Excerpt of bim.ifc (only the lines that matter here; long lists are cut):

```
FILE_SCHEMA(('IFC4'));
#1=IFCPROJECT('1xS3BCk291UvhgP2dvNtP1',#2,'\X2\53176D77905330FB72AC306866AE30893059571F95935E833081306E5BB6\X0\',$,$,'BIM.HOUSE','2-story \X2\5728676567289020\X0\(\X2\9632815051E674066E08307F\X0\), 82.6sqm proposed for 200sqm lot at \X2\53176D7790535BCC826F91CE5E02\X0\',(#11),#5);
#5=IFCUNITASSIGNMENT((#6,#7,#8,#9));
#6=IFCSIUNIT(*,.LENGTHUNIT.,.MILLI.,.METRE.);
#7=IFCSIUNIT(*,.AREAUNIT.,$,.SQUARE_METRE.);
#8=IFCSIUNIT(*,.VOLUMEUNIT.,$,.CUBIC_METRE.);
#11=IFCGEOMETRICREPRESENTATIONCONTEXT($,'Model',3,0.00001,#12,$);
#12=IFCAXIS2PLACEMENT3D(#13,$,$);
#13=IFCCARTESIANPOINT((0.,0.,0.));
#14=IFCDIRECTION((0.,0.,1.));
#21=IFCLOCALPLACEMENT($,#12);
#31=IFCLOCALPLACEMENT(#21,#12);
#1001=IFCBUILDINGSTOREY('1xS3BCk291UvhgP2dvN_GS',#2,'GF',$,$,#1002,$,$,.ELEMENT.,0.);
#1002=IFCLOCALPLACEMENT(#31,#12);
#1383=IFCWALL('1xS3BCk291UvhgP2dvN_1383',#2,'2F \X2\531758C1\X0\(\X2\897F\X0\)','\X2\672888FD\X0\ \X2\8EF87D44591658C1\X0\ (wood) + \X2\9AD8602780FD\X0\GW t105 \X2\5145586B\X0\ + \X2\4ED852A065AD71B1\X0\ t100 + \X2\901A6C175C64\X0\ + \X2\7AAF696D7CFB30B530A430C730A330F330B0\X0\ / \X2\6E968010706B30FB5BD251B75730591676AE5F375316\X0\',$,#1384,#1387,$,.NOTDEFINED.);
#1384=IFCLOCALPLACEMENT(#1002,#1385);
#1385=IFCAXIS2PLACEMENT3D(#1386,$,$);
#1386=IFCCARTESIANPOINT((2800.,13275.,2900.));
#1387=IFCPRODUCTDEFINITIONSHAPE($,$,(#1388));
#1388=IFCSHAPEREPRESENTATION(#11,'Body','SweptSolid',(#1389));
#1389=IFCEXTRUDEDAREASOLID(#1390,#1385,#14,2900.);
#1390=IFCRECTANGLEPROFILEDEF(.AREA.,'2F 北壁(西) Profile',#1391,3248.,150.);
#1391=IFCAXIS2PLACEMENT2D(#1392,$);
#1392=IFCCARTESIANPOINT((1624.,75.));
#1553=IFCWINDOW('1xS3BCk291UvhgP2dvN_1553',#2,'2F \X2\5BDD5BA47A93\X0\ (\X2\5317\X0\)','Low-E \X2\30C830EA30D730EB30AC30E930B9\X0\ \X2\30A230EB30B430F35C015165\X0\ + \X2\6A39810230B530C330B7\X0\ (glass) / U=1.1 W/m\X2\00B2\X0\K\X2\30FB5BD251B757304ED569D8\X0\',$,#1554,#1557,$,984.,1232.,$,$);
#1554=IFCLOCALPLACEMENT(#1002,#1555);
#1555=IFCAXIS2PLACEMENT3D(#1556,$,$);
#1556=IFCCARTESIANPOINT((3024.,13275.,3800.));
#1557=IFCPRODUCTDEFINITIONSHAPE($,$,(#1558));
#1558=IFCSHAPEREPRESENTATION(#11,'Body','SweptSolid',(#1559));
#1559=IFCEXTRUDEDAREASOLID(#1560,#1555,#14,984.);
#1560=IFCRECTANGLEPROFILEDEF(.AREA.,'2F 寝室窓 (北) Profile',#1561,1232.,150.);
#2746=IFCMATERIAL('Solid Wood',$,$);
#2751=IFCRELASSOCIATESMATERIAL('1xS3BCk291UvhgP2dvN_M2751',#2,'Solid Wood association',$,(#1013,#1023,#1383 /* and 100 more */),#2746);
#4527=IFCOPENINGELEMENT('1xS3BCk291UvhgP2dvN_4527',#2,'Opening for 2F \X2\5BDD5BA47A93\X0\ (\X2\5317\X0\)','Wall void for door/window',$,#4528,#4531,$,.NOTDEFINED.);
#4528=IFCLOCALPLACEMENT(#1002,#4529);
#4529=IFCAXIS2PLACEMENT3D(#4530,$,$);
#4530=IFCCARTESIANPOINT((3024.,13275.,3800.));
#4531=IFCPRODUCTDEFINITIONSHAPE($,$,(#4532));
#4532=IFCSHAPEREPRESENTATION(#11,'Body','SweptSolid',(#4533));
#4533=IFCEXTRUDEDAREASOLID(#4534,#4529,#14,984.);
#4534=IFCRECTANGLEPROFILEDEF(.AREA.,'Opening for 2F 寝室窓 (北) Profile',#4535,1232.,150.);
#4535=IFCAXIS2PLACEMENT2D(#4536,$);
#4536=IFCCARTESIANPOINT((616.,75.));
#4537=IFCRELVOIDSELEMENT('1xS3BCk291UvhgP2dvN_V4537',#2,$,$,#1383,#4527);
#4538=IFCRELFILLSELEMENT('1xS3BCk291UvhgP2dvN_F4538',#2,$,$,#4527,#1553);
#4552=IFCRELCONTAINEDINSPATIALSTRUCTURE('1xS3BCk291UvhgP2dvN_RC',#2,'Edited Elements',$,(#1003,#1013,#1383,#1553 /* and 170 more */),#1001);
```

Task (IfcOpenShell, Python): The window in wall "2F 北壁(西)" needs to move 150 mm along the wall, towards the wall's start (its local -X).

```python
import ifcopenshell
import ifcopenshell.api.geometry
import ifcopenshell.util.placement
import ifcopenshell.util.unit

model = ifcopenshell.open("bim.ifc")
unit_scale = ifcopenshell.util.unit.calculate_unit_scale(model)

window = model.by_id(1553)
opening = window.FillsVoids[0].RelatingOpeningElement
wall = opening.VoidsElements[0].RelatingBuildingElement

wall_matrix = ifcopenshell.util.placement.get_local_placement(wall.ObjectPlacement)
shift = wall_matrix[:3, 0] * -0.15 / unit_scale
before = ifcopenshell.util.placement.get_local_placement(window.ObjectPlacement)[:3, 3].copy()

# The window is not placed relative to its opening, so move both.
for product in (opening, window):
    matrix = ifcopenshell.util.placement.get_local_placement(product.ObjectPlacement)
    matrix[:3, 3] += shift
    ifcopenshell.api.geometry.edit_object_placement(model, product=product, matrix=matrix, is_si=False)

after = ifcopenshell.util.placement.get_local_placement(window.ObjectPlacement)[:3, 3]
print("window moved by", (after - before).round(3) + 0.0)

model.write("bim_updated.ifc")
```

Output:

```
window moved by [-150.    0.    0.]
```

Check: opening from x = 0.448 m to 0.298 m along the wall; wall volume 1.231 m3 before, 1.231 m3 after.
